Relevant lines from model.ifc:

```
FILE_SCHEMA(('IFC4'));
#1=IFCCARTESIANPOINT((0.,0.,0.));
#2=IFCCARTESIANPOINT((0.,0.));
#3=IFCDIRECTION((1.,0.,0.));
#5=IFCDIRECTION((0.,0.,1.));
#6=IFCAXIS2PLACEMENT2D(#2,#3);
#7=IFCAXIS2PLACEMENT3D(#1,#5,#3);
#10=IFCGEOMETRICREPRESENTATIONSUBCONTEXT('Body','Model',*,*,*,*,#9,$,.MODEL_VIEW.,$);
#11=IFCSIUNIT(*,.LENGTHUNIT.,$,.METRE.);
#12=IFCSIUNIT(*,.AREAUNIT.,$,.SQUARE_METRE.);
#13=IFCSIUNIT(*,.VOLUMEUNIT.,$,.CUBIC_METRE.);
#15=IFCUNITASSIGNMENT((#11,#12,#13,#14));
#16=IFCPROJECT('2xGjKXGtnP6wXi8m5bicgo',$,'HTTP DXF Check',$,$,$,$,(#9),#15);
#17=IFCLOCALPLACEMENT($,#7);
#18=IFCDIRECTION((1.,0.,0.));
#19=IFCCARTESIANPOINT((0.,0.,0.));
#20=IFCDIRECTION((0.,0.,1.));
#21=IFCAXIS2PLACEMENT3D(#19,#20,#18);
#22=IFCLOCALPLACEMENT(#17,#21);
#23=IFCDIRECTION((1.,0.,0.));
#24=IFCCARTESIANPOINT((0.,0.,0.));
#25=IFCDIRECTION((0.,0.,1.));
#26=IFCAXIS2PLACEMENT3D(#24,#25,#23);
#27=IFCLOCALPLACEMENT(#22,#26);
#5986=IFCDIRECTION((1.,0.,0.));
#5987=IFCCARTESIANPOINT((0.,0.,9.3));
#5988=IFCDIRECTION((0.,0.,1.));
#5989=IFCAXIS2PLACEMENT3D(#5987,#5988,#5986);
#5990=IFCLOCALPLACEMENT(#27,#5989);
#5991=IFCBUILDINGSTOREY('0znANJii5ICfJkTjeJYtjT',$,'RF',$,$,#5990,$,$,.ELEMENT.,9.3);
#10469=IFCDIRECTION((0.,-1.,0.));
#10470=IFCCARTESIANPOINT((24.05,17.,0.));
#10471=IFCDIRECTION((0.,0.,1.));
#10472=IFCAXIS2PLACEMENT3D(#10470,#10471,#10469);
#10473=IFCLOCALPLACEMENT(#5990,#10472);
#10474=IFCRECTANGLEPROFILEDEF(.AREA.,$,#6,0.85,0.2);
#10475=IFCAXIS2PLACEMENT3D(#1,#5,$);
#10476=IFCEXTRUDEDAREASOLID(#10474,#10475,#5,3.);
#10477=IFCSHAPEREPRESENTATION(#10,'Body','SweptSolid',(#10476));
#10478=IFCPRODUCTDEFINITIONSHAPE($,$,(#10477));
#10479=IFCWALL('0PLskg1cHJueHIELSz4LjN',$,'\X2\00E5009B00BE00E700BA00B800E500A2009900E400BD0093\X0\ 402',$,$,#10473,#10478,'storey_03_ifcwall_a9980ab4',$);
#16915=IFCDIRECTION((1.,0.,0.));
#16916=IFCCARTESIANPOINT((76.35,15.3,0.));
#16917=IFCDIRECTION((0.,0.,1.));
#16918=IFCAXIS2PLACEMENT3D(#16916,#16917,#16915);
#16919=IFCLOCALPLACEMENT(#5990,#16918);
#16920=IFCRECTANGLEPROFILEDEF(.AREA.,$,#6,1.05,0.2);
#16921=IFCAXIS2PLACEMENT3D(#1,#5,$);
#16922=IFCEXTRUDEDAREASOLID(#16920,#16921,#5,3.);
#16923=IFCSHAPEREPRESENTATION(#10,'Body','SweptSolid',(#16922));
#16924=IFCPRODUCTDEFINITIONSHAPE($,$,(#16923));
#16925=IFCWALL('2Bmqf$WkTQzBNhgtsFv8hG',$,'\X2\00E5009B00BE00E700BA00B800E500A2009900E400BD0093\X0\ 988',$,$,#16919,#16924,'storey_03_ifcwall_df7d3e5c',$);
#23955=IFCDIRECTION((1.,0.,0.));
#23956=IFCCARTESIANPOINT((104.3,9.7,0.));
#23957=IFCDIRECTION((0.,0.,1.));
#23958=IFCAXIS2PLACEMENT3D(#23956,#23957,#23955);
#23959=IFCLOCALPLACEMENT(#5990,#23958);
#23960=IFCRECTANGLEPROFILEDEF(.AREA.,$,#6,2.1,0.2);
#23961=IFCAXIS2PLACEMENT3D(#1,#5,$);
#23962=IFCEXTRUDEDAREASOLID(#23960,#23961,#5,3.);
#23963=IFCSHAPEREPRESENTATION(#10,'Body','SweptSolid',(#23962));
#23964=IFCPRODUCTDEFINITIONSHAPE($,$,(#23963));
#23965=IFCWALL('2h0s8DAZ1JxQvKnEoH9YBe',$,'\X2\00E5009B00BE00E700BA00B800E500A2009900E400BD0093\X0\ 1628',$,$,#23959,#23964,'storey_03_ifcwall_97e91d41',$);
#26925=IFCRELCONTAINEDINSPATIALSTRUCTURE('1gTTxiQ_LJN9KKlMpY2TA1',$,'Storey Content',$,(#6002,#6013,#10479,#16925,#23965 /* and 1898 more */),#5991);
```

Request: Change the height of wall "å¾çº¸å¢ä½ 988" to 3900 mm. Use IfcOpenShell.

```python
import ifcopenshell
import ifcopenshell.geom
import ifcopenshell.util.representation
import ifcopenshell.util.shape

model = ifcopenshell.open("model.ifc")
settings = ifcopenshell.geom.settings()


def volume(element):
    """Net volume in cubic metres, openings subtracted."""
    shape = ifcopenshell.geom.create_shape(settings, element)
    return ifcopenshell.util.shape.get_volume(shape.geometry)


wall = model.by_guid("2Bmqf$WkTQzBNhgtsFv8hG")
before = volume(wall)

body = ifcopenshell.util.representation.get_representation(wall, "Model", "Body")
solid = body.Items[0]
old_height = solid.Depth
solid.Depth = 3.9
after = volume(wall)

print(f"height {old_height:g} -> {solid.Depth:g}, volume {before:.3f} -> {after:.3f} m3")

model.write("model-out.ifc")
```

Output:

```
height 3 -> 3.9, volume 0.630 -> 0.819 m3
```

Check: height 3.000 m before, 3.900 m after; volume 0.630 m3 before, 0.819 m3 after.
